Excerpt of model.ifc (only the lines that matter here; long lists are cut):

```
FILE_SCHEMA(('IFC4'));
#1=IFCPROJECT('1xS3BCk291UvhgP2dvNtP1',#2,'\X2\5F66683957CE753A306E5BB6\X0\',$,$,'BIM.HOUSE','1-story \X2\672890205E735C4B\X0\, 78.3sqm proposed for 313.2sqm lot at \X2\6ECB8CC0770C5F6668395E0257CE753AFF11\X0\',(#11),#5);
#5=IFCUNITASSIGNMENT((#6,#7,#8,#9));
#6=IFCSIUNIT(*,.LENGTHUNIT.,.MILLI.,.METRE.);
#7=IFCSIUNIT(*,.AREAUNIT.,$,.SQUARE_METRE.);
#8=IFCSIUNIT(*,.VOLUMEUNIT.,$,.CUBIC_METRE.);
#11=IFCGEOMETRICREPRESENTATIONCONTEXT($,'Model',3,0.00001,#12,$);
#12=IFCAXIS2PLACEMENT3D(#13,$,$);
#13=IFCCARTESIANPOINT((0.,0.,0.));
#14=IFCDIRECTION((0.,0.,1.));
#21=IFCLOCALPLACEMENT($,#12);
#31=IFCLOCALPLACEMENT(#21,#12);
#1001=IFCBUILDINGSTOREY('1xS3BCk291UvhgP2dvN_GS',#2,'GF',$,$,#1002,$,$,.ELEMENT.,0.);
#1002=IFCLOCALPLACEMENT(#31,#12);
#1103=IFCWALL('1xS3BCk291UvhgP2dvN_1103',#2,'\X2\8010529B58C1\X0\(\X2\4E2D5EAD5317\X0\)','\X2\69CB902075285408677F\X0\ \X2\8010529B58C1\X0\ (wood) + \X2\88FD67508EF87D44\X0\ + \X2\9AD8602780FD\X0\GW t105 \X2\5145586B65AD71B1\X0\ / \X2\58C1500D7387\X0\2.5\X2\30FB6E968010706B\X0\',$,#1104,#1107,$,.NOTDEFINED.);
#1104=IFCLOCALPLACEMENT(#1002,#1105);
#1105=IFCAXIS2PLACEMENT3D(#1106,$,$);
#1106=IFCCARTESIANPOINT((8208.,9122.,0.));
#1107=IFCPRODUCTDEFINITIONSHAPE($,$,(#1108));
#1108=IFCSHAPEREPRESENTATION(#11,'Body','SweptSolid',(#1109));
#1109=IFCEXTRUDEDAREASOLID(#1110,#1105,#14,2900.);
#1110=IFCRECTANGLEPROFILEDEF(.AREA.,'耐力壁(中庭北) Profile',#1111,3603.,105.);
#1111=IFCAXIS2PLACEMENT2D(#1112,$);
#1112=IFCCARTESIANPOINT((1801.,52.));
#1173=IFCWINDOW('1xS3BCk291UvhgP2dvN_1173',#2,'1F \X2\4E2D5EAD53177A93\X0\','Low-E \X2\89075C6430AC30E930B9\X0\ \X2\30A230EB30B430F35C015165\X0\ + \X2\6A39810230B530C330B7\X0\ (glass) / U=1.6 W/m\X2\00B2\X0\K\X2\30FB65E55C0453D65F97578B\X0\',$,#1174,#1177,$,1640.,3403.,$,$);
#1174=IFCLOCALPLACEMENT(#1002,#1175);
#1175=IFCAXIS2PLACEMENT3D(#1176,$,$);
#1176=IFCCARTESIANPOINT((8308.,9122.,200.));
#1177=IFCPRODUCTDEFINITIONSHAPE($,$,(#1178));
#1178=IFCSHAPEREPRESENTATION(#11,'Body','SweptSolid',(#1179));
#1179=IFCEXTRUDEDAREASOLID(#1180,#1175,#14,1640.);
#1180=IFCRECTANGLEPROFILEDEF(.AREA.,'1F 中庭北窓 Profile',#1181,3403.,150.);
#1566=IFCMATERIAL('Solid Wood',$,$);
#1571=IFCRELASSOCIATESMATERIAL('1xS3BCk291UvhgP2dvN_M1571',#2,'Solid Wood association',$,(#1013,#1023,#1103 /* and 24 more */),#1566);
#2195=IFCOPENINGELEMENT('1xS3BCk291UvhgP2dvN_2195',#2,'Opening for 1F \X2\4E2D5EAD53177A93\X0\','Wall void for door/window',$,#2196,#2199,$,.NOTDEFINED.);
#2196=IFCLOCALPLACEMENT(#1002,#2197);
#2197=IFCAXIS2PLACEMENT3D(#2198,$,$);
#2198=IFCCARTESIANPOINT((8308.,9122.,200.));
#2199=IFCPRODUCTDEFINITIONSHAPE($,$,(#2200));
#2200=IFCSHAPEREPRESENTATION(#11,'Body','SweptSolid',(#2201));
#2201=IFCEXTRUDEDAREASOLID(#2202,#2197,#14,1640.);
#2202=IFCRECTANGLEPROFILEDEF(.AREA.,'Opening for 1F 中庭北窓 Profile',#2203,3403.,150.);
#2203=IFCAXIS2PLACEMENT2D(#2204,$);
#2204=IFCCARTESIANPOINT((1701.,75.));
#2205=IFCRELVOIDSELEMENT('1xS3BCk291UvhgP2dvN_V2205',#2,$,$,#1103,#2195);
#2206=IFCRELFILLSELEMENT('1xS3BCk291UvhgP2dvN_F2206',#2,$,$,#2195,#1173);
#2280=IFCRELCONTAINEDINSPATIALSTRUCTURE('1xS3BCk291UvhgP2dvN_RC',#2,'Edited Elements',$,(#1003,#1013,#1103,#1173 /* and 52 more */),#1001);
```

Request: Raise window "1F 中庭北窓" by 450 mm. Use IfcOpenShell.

```python
import numpy as np
import ifcopenshell
import ifcopenshell.api.geometry
import ifcopenshell.util.placement
import ifcopenshell.util.unit

model = ifcopenshell.open("model.ifc")
unit_scale = ifcopenshell.util.unit.calculate_unit_scale(model)

window = model.by_guid("1xS3BCk291UvhgP2dvN_1173")
opening = window.FillsVoids[0].RelatingOpeningElement
dz = 0.45 / unit_scale

shift = np.array([0.0, 0.0, dz])
# The window is not placed relative to its opening, so move both.
for product in (opening, window):
    matrix = ifcopenshell.util.placement.get_local_placement(product.ObjectPlacement)
    matrix[:3, 3] += shift
    ifcopenshell.api.geometry.edit_object_placement(model, product=product, matrix=matrix, is_si=False)

print(f"moved by {dz * unit_scale:+.3f} m")

model.write("model_rev.ifc")
```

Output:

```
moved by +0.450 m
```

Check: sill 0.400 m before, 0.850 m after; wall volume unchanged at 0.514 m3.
